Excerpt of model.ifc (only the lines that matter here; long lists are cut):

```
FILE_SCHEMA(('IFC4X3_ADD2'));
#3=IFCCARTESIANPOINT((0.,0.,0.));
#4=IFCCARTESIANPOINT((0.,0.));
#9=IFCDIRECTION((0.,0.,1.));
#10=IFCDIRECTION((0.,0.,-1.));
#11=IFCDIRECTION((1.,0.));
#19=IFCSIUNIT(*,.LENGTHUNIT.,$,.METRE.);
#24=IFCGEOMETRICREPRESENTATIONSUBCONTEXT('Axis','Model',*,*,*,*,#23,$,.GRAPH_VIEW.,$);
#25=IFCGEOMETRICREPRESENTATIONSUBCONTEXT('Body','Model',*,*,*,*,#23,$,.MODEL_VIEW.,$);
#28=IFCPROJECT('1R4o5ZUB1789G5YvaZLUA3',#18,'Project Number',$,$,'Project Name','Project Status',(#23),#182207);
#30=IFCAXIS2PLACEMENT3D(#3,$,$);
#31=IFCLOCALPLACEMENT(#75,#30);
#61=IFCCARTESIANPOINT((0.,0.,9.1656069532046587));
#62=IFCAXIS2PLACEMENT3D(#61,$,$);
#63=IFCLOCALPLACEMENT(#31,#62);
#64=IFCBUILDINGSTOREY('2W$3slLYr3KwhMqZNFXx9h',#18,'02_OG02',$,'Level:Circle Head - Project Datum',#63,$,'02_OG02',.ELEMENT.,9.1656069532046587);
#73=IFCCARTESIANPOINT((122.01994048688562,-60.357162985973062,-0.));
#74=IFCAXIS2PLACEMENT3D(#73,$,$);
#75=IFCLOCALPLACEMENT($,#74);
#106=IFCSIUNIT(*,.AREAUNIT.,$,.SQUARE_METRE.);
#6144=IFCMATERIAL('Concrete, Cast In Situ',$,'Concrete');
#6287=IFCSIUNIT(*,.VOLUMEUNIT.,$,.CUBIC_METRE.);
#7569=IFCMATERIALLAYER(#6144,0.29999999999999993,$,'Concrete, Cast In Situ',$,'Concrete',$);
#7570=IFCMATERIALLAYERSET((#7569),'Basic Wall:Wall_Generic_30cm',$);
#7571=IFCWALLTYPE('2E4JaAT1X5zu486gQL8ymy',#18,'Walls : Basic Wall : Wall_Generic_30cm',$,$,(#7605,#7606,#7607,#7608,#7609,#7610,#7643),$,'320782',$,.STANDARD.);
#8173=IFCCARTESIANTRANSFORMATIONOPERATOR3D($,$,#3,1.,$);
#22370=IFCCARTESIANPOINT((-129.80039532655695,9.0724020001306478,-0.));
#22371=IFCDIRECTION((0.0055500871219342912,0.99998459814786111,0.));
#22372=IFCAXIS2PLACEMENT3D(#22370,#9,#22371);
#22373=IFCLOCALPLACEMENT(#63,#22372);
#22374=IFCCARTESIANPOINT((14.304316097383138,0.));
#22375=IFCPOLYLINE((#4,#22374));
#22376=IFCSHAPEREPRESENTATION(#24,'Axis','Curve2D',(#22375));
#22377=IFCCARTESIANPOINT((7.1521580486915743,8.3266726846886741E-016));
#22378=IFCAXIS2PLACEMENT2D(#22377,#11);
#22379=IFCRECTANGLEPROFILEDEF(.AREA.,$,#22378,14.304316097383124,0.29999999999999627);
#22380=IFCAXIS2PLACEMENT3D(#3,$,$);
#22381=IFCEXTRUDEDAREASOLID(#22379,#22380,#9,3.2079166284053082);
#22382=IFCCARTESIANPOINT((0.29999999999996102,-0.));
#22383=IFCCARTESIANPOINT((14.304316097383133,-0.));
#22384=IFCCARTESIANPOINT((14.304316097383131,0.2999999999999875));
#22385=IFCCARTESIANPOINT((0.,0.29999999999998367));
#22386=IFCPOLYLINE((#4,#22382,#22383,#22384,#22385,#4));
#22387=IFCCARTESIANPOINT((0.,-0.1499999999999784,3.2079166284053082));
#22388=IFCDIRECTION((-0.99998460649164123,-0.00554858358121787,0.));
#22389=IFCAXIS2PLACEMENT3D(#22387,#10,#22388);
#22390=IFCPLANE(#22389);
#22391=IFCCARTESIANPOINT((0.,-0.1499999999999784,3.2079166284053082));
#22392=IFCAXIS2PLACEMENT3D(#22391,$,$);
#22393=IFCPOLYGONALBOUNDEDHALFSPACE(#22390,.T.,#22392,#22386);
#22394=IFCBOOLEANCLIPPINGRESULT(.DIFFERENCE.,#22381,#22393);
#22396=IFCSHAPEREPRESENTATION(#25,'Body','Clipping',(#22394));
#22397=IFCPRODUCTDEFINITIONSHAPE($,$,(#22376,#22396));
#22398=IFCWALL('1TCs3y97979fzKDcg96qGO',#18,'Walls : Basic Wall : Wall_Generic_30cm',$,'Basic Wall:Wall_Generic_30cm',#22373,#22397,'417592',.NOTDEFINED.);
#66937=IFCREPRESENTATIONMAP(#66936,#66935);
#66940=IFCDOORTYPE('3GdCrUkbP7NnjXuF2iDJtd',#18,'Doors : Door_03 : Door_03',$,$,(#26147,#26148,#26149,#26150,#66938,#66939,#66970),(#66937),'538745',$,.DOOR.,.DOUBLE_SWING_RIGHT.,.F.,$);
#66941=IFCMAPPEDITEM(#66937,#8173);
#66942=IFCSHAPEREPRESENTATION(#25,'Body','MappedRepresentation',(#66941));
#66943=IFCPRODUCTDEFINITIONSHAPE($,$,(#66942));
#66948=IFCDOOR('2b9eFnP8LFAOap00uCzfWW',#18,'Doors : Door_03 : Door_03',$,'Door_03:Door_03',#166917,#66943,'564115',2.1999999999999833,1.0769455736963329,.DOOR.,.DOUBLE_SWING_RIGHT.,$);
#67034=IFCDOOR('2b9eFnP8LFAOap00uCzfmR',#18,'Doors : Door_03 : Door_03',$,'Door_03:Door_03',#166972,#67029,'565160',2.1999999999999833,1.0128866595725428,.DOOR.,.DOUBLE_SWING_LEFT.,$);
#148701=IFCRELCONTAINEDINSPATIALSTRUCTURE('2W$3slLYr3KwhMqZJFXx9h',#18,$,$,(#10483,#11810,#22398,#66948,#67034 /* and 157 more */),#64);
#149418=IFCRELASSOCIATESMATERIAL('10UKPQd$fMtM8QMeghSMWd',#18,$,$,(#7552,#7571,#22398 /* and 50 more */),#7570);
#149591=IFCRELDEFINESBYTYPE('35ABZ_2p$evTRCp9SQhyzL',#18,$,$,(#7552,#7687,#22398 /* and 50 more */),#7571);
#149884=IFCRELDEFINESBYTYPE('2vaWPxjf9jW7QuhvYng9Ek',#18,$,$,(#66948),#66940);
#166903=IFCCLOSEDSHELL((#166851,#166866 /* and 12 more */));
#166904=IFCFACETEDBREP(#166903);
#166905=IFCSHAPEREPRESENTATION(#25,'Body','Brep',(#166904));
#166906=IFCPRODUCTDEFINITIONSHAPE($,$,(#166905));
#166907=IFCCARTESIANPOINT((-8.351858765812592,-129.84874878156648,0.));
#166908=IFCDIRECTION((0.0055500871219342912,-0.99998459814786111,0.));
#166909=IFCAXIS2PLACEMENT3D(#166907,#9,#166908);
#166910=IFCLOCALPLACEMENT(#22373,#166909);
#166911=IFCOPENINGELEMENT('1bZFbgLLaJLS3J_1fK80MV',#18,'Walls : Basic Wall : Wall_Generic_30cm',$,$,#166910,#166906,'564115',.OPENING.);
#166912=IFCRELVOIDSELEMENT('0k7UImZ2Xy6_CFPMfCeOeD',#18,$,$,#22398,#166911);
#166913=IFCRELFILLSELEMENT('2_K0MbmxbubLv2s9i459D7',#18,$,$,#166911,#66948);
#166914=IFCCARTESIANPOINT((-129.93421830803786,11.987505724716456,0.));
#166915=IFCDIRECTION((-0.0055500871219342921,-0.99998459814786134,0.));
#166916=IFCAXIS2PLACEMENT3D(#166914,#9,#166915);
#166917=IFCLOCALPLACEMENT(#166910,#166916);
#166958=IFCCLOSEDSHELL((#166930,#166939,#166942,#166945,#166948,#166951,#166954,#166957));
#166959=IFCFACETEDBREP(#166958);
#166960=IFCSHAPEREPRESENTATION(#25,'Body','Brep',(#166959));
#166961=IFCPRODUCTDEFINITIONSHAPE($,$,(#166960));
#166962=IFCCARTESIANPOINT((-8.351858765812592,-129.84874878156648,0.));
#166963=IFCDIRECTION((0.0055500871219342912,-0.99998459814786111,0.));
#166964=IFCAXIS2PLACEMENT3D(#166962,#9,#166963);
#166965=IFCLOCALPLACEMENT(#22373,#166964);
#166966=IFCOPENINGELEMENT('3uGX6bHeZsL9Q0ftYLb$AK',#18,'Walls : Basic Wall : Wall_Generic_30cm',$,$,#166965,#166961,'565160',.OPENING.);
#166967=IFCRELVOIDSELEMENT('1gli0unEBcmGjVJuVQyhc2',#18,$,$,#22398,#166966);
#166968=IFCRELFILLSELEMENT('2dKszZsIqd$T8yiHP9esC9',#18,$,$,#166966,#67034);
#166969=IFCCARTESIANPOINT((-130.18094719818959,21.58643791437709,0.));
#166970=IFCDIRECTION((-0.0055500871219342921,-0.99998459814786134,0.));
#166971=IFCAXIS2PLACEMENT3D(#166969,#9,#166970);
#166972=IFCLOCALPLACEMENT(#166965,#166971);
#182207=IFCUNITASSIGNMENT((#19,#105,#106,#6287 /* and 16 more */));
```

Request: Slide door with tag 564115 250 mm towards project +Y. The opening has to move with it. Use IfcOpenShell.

```python
import ifcopenshell
import ifcopenshell.api.geometry
import ifcopenshell.util.placement

model = ifcopenshell.open("model.ifc")

door = model.by_guid("2b9eFnP8LFAOap00uCzfWW")
opening = door.FillsVoids[0].RelatingOpeningElement
wall = opening.VoidsElements[0].RelatingBuildingElement

wall_matrix = ifcopenshell.util.placement.get_local_placement(wall.ObjectPlacement)
shift = wall_matrix[:3, 0] * 0.25
before = ifcopenshell.util.placement.get_local_placement(door.ObjectPlacement)[:3, 3].copy()

# The door is placed relative to its opening, so it follows when the opening moves.
matrix = ifcopenshell.util.placement.get_local_placement(opening.ObjectPlacement)
matrix[:3, 3] += shift
ifcopenshell.api.geometry.edit_object_placement(
    model, product=opening, matrix=matrix, is_si=False, should_transform_children=True
)

after = ifcopenshell.util.placement.get_local_placement(door.ObjectPlacement)[:3, 3]
print("door moved by", (after - before).round(3) + 0.0)

model.write("model-out.ifc")
```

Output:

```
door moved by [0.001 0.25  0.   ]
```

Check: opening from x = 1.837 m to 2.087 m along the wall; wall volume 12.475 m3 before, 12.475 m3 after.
